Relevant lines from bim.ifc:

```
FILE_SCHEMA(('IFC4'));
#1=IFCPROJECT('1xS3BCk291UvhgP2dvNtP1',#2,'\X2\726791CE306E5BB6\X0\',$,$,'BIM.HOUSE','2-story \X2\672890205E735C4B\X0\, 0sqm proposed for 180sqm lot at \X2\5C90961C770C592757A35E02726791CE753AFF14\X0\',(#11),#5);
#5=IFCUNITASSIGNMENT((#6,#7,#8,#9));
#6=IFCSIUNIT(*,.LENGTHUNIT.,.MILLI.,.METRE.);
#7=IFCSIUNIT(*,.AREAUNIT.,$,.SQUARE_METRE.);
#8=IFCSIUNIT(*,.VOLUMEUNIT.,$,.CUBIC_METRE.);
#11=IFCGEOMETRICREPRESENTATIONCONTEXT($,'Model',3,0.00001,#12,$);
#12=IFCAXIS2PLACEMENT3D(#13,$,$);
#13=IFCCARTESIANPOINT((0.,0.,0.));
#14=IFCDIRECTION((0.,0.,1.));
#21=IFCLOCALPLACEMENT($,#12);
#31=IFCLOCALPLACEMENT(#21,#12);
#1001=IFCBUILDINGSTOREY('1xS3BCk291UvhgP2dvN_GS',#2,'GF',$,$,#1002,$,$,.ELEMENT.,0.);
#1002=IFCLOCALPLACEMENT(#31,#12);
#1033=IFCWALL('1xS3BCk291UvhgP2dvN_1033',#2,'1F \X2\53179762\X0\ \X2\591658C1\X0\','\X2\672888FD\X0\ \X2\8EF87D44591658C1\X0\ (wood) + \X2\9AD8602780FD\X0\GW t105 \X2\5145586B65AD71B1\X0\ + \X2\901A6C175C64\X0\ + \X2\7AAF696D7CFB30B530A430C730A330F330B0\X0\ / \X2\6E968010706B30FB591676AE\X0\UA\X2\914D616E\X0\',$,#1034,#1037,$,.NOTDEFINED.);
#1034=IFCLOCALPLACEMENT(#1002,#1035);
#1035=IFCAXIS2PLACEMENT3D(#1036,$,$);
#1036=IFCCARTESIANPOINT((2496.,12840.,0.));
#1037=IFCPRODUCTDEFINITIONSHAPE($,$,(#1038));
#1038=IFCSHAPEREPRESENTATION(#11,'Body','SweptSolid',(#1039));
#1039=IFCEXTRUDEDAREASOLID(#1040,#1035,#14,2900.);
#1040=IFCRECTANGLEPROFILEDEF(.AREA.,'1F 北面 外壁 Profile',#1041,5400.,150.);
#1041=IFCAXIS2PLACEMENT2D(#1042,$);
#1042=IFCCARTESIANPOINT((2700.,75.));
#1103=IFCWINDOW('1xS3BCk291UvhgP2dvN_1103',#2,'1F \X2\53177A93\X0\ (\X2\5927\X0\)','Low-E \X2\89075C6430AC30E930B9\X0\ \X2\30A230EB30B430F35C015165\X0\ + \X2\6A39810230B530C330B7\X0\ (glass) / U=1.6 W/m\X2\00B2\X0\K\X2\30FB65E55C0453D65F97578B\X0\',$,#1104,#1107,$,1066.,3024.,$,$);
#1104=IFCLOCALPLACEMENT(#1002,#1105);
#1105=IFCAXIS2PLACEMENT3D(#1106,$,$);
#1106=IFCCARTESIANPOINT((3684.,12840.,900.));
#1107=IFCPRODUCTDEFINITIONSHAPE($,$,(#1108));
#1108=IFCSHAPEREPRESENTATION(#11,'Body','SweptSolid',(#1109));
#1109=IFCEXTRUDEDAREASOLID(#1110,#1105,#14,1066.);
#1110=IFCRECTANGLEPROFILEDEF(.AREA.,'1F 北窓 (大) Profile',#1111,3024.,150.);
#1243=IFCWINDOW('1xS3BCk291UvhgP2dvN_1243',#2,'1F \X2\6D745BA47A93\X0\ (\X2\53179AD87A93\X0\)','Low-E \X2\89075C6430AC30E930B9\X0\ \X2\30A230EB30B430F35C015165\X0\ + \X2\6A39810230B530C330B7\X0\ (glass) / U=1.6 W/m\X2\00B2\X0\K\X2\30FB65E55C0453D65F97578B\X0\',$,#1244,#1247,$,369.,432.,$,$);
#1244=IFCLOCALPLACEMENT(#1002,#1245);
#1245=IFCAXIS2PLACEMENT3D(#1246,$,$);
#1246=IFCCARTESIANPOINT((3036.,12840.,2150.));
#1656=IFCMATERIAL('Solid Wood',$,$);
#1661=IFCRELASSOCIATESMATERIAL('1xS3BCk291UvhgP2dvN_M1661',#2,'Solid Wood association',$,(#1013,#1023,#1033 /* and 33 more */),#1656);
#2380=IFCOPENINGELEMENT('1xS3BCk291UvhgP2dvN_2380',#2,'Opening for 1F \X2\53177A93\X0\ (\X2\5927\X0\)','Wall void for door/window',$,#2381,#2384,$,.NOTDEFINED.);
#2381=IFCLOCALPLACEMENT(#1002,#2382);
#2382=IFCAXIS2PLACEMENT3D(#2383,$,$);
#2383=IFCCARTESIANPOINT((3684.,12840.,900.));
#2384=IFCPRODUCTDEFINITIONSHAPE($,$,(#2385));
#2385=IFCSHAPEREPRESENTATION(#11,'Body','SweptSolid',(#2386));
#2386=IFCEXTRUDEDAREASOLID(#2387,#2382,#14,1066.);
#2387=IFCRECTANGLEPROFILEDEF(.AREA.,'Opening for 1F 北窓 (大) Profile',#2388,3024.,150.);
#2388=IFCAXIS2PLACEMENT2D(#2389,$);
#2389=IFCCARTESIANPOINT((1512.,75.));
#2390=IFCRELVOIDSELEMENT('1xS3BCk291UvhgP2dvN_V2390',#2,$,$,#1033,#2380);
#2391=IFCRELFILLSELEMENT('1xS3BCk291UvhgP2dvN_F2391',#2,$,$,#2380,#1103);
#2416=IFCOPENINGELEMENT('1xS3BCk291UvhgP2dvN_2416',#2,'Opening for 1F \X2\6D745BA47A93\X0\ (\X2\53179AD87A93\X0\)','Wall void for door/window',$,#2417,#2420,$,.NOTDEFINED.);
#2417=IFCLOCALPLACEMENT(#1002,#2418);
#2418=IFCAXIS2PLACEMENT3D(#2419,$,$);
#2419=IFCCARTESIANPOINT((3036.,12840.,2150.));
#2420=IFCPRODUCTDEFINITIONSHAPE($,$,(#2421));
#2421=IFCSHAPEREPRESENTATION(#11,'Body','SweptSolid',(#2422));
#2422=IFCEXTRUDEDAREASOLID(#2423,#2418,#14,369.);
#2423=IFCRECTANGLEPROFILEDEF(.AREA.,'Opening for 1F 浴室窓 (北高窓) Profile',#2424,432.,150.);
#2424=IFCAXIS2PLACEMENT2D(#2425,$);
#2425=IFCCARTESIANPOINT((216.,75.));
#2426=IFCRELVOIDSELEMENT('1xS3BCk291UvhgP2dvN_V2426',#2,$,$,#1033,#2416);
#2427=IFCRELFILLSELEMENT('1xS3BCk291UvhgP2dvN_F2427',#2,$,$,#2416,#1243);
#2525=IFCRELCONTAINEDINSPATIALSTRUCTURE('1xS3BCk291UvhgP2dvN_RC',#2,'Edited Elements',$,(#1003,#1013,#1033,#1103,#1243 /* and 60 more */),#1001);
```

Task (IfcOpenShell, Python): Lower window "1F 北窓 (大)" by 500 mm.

```python
import numpy as np
import ifcopenshell
import ifcopenshell.api.geometry
import ifcopenshell.util.placement
import ifcopenshell.util.unit

model = ifcopenshell.open("bim.ifc")
unit_scale = ifcopenshell.util.unit.calculate_unit_scale(model)

window = model.by_guid("1xS3BCk291UvhgP2dvN_1103")
opening = window.FillsVoids[0].RelatingOpeningElement
dz = -0.5 / unit_scale

shift = np.array([0.0, 0.0, dz])
# The window is not placed relative to its opening, so move both.
for product in (opening, window):
    matrix = ifcopenshell.util.placement.get_local_placement(product.ObjectPlacement)
    matrix[:3, 3] += shift
    ifcopenshell.api.geometry.edit_object_placement(model, product=product, matrix=matrix, is_si=False)

print(f"moved by {dz * unit_scale:+.3f} m")

model.write("bim_rev.ifc")
```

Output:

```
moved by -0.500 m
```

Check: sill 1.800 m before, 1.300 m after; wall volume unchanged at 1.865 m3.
